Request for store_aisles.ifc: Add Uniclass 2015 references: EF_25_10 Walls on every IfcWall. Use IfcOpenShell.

First a look at what the model holds.

```python
import ifcopenshell

model = ifcopenshell.open("store_aisles.ifc")
print(model.schema)
print("classifications:", [c.Name for c in model.by_type("IfcClassification")])
for ifc_class in ("IfcDoor", "IfcRoof", "IfcStair", "IfcWall", "IfcWindow"):
    print(ifc_class, len(model.by_type(ifc_class)))
```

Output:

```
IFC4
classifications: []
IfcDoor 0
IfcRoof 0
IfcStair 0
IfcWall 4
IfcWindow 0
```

```python
import ifcopenshell
import ifcopenshell.api.classification

model = ifcopenshell.open("store_aisles.ifc")

system = ifcopenshell.api.classification.add_classification(model, classification="Uniclass 2015")

codes = {
    "IfcWall": ("EF_25_10", "Walls"),
}
for ifc_class, (code, name) in codes.items():
    products = model.by_type(ifc_class)
    ifcopenshell.api.classification.add_reference(
        model, products=products, classification=system, identification=code, name=name
    )
    print(code, len(products))

model.write("store_aisles_updated.ifc")
```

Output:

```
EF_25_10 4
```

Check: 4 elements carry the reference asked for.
